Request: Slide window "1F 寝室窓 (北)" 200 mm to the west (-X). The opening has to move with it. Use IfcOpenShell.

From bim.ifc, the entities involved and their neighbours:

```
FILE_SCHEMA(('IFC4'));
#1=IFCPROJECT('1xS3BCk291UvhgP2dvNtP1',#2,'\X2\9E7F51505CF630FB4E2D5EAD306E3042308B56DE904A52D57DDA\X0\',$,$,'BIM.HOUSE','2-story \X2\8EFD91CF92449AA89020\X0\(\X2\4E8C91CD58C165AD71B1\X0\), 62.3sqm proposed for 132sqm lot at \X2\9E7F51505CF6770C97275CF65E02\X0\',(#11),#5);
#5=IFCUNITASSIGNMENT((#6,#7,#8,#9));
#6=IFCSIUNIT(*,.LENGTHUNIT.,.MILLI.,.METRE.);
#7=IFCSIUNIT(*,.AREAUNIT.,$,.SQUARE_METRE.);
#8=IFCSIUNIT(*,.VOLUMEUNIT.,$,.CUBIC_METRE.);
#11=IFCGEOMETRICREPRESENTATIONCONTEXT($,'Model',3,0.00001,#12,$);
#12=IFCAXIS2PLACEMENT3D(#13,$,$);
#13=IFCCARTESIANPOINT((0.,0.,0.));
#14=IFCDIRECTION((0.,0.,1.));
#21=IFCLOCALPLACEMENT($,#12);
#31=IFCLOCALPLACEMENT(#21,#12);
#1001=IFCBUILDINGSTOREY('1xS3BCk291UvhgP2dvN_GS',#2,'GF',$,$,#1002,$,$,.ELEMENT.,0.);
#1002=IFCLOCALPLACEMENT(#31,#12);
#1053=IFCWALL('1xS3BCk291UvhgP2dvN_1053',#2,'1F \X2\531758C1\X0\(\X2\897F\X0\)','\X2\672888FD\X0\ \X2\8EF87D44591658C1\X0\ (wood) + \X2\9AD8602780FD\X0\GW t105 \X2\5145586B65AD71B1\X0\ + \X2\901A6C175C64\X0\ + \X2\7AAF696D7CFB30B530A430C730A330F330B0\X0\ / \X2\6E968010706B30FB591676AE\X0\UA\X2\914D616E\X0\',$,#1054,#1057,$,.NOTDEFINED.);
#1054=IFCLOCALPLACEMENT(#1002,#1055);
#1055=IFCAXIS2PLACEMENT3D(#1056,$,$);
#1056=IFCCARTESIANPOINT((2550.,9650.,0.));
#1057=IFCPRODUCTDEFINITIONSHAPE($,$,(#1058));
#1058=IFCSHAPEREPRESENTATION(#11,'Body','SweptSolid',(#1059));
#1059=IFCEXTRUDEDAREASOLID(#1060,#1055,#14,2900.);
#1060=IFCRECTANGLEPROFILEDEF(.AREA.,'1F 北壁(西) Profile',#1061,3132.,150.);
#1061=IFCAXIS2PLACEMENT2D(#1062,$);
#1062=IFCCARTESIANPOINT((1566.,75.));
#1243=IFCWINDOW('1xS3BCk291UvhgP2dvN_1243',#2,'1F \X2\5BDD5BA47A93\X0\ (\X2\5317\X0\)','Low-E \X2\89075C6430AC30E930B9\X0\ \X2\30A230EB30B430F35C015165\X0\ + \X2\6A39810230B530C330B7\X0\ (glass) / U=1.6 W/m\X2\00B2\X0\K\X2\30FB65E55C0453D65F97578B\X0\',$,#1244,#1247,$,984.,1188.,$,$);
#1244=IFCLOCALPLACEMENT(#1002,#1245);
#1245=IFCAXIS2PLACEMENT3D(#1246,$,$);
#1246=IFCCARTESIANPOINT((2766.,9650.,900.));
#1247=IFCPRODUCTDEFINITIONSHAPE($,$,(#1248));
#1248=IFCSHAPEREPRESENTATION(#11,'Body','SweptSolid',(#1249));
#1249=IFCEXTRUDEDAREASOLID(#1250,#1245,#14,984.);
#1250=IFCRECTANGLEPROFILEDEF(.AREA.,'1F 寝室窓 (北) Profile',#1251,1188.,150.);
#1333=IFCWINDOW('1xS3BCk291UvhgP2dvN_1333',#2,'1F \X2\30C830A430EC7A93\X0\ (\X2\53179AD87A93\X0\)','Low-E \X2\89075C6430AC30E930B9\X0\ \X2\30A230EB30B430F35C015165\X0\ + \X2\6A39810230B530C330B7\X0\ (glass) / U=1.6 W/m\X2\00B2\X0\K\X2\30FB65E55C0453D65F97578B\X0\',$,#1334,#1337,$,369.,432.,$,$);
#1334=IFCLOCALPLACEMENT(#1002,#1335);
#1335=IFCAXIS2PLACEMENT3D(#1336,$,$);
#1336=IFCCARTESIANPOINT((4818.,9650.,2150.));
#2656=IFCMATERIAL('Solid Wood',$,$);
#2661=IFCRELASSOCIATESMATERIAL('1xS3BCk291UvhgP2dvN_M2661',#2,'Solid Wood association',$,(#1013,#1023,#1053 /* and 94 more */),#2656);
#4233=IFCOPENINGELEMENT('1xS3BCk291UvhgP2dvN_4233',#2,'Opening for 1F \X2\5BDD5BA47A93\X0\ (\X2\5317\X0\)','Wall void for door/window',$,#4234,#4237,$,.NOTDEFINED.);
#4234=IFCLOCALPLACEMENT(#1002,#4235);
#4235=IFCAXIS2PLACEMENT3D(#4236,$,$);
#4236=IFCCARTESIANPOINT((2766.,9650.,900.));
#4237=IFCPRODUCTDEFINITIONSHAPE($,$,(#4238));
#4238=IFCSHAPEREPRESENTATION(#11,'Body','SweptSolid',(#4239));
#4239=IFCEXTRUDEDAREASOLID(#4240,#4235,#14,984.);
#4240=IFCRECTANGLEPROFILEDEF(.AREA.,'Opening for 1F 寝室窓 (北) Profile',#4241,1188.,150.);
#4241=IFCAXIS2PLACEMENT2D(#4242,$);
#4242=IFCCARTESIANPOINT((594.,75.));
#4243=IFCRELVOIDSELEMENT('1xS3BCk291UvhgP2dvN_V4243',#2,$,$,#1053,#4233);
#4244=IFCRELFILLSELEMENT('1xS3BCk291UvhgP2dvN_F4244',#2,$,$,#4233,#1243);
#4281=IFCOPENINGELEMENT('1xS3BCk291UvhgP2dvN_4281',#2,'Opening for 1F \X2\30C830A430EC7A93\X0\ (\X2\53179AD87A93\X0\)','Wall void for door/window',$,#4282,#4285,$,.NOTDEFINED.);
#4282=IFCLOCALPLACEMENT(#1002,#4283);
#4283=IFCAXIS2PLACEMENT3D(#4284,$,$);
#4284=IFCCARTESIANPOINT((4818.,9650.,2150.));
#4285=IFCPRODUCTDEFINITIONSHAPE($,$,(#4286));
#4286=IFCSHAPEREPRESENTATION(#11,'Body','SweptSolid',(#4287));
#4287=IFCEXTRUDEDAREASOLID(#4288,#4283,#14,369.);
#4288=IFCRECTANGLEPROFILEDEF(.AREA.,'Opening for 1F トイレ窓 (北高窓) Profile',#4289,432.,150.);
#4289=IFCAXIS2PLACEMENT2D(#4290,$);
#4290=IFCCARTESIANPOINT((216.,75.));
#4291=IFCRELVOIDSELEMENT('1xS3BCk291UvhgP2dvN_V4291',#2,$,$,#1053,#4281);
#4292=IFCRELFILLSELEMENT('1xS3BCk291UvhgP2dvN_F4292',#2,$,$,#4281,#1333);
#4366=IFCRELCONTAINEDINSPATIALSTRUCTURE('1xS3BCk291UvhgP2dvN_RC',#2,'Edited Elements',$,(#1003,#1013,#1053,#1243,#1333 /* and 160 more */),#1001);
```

```python
import ifcopenshell
import ifcopenshell.api.geometry
import ifcopenshell.util.placement
import ifcopenshell.util.unit

model = ifcopenshell.open("bim.ifc")
unit_scale = ifcopenshell.util.unit.calculate_unit_scale(model)

window = model.by_guid("1xS3BCk291UvhgP2dvN_1243")
opening = window.FillsVoids[0].RelatingOpeningElement
wall = opening.VoidsElements[0].RelatingBuildingElement

wall_matrix = ifcopenshell.util.placement.get_local_placement(wall.ObjectPlacement)
shift = wall_matrix[:3, 0] * -0.2 / unit_scale
before = ifcopenshell.util.placement.get_local_placement(window.ObjectPlacement)[:3, 3].copy()

# The window is not placed relative to its opening, so move both.
for product in (opening, window):
    matrix = ifcopenshell.util.placement.get_local_placement(product.ObjectPlacement)
    matrix[:3, 3] += shift
    ifcopenshell.api.geometry.edit_object_placement(model, product=product, matrix=matrix, is_si=False)

after = ifcopenshell.util.placement.get_local_placement(window.ObjectPlacement)[:3, 3]
print("window moved by", (after - before).round(3) + 0.0)

model.write("bim_rev.ifc")
```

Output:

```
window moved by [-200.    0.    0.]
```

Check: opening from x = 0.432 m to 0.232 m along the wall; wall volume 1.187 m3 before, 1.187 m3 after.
